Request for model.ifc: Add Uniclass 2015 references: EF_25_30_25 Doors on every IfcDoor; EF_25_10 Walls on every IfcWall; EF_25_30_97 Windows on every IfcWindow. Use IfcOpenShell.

First a look at what the model holds.

```python
import ifcopenshell

model = ifcopenshell.open("model.ifc")
print(model.schema)
print("classifications:", [c.Name for c in model.by_type("IfcClassification")])
for ifc_class in ("IfcDoor", "IfcRoof", "IfcStair", "IfcWall", "IfcWindow"):
    print(ifc_class, len(model.by_type(ifc_class)))
```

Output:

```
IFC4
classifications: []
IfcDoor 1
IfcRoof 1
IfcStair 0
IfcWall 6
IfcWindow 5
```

```python
import ifcopenshell
import ifcopenshell.api.classification

model = ifcopenshell.open("model.ifc")

system = ifcopenshell.api.classification.add_classification(model, classification="Uniclass 2015")

codes = {
    "IfcDoor": ("EF_25_30_25", "Doors"),
    "IfcWall": ("EF_25_10", "Walls"),
    "IfcWindow": ("EF_25_30_97", "Windows"),
}
for ifc_class, (code, name) in codes.items():
    products = model.by_type(ifc_class)
    ifcopenshell.api.classification.add_reference(
        model, products=products, classification=system, identification=code, name=name
    )
    print(code, len(products))

model.write("model_updated.ifc")
```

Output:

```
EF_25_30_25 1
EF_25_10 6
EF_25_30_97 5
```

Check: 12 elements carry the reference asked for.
